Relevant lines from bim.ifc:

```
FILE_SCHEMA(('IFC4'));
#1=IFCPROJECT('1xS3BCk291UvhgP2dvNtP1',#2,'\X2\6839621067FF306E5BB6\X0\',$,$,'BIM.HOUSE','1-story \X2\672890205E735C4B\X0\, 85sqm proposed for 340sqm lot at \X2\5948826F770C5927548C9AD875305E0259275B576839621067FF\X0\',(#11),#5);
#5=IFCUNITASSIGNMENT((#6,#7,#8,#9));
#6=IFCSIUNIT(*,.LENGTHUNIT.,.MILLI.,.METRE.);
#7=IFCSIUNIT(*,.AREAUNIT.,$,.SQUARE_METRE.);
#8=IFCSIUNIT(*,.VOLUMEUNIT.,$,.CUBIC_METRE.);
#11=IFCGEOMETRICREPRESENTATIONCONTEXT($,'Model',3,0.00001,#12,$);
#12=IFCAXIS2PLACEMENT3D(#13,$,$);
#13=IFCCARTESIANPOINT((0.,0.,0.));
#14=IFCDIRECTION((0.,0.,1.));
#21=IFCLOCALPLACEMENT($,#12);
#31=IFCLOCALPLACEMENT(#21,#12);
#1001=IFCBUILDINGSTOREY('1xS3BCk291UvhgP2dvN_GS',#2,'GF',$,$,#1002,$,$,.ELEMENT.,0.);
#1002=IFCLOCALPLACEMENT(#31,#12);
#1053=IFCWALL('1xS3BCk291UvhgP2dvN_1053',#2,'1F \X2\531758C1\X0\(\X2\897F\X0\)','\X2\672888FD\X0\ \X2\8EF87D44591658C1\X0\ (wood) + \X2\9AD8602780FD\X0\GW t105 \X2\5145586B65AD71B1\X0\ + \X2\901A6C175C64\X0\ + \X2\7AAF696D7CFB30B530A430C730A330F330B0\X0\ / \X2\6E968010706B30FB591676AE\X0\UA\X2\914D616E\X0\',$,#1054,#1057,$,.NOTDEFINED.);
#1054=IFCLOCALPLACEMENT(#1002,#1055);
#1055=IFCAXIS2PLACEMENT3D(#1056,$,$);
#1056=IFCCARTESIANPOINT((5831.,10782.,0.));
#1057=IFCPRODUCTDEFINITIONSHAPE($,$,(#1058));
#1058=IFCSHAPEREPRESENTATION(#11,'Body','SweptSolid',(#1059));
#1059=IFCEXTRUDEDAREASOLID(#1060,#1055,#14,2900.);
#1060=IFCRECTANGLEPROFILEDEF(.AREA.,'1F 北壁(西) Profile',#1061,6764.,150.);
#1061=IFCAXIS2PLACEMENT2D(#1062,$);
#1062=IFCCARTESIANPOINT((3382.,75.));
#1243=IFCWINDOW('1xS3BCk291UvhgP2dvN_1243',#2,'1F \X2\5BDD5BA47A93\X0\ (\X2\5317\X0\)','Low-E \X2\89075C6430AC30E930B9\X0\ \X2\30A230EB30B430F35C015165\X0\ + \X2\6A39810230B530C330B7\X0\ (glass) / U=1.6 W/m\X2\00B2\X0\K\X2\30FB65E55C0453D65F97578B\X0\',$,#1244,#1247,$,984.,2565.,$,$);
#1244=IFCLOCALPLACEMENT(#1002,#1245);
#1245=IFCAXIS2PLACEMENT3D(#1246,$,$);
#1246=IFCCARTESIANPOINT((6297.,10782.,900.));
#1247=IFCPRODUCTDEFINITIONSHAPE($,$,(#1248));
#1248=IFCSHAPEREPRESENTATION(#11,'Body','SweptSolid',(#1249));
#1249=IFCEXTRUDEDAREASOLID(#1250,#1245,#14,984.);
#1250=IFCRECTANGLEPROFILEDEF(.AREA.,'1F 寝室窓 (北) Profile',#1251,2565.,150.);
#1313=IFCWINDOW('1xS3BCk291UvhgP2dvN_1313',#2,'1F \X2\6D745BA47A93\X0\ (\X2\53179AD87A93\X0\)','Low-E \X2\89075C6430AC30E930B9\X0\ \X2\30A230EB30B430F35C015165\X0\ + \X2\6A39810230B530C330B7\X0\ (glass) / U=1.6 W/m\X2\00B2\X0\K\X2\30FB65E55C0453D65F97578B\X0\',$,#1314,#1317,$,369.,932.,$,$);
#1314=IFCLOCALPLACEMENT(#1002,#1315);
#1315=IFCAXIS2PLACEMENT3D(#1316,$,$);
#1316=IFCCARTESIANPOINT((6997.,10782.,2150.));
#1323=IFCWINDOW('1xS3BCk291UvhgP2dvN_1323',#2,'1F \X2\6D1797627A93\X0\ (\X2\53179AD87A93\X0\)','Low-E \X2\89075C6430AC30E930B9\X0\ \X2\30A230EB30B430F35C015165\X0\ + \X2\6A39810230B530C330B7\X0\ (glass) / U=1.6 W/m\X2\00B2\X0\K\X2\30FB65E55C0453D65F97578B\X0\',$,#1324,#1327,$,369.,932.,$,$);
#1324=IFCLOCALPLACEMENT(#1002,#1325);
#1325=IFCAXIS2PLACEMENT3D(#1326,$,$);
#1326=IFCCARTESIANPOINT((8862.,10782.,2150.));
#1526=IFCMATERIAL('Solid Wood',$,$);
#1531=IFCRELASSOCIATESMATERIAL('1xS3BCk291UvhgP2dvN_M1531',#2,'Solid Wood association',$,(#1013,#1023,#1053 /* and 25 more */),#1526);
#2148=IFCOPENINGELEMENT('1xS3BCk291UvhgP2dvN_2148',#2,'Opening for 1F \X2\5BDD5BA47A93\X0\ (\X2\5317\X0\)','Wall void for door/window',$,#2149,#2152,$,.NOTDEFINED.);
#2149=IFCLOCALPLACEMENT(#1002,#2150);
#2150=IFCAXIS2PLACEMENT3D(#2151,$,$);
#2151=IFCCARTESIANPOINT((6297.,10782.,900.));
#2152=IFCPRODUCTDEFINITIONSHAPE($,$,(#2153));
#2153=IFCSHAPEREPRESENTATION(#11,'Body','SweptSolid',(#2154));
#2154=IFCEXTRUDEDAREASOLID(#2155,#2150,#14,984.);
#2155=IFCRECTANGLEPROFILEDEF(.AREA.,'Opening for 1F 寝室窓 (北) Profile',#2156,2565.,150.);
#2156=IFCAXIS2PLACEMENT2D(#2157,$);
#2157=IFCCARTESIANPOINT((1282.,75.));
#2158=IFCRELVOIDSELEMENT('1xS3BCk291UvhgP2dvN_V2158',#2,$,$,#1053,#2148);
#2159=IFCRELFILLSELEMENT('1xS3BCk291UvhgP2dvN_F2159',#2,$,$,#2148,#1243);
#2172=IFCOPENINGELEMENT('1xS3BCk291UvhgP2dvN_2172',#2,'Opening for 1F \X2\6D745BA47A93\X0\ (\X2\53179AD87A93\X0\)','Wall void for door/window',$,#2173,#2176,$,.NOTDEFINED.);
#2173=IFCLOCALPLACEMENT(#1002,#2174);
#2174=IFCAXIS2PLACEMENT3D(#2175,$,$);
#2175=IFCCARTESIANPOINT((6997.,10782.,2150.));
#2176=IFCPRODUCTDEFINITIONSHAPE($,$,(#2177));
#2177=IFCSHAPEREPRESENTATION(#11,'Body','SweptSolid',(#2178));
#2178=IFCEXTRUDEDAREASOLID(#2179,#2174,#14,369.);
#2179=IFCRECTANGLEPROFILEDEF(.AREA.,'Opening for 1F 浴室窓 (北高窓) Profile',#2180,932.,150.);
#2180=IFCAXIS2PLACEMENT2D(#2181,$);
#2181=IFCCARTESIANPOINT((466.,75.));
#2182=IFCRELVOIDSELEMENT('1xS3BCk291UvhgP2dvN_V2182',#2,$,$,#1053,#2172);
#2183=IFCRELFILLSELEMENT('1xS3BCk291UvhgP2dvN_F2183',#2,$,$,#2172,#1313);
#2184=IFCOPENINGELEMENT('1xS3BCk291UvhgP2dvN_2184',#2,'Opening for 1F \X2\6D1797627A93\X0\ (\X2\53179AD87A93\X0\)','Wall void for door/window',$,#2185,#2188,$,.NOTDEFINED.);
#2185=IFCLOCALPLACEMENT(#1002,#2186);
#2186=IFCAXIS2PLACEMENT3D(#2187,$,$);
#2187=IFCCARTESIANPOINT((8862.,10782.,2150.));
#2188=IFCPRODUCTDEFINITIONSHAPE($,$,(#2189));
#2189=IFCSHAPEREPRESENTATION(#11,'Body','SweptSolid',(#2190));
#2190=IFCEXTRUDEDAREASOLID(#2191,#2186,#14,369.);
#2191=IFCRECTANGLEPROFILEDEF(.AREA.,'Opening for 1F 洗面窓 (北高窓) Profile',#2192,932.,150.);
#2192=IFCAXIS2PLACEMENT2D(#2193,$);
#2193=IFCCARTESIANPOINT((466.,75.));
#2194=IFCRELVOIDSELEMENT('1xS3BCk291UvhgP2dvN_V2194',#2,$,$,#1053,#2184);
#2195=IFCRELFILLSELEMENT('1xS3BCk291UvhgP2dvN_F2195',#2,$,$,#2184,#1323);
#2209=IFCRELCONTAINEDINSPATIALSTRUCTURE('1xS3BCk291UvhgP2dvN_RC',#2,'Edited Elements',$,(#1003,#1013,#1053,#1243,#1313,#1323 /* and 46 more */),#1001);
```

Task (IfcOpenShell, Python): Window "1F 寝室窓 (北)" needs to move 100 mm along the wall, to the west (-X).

```python
import ifcopenshell
import ifcopenshell.api.geometry
import ifcopenshell.util.placement

model = ifcopenshell.open("bim.ifc")

window = model.by_id(1243)
opening = window.FillsVoids[0].RelatingOpeningElement
wall = opening.VoidsElements[0].RelatingBuildingElement

wall_matrix = ifcopenshell.util.placement.get_local_placement(wall.ObjectPlacement)
shift = wall_matrix[:3, 0] * -100.0
before = ifcopenshell.util.placement.get_local_placement(window.ObjectPlacement)[:3, 3].copy()

# The window is not placed relative to its opening, so move both.
for product in (opening, window):
    matrix = ifcopenshell.util.placement.get_local_placement(product.ObjectPlacement)
    matrix[:3, 3] += shift
    ifcopenshell.api.geometry.edit_object_placement(model, product=product, matrix=matrix, is_si=False)

after = ifcopenshell.util.placement.get_local_placement(window.ObjectPlacement)[:3, 3]
print("window moved by", (after - before).round(3) + 0.0)

model.write("bim_edited.ifc")
```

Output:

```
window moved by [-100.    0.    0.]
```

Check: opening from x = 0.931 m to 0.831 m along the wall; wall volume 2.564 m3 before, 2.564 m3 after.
